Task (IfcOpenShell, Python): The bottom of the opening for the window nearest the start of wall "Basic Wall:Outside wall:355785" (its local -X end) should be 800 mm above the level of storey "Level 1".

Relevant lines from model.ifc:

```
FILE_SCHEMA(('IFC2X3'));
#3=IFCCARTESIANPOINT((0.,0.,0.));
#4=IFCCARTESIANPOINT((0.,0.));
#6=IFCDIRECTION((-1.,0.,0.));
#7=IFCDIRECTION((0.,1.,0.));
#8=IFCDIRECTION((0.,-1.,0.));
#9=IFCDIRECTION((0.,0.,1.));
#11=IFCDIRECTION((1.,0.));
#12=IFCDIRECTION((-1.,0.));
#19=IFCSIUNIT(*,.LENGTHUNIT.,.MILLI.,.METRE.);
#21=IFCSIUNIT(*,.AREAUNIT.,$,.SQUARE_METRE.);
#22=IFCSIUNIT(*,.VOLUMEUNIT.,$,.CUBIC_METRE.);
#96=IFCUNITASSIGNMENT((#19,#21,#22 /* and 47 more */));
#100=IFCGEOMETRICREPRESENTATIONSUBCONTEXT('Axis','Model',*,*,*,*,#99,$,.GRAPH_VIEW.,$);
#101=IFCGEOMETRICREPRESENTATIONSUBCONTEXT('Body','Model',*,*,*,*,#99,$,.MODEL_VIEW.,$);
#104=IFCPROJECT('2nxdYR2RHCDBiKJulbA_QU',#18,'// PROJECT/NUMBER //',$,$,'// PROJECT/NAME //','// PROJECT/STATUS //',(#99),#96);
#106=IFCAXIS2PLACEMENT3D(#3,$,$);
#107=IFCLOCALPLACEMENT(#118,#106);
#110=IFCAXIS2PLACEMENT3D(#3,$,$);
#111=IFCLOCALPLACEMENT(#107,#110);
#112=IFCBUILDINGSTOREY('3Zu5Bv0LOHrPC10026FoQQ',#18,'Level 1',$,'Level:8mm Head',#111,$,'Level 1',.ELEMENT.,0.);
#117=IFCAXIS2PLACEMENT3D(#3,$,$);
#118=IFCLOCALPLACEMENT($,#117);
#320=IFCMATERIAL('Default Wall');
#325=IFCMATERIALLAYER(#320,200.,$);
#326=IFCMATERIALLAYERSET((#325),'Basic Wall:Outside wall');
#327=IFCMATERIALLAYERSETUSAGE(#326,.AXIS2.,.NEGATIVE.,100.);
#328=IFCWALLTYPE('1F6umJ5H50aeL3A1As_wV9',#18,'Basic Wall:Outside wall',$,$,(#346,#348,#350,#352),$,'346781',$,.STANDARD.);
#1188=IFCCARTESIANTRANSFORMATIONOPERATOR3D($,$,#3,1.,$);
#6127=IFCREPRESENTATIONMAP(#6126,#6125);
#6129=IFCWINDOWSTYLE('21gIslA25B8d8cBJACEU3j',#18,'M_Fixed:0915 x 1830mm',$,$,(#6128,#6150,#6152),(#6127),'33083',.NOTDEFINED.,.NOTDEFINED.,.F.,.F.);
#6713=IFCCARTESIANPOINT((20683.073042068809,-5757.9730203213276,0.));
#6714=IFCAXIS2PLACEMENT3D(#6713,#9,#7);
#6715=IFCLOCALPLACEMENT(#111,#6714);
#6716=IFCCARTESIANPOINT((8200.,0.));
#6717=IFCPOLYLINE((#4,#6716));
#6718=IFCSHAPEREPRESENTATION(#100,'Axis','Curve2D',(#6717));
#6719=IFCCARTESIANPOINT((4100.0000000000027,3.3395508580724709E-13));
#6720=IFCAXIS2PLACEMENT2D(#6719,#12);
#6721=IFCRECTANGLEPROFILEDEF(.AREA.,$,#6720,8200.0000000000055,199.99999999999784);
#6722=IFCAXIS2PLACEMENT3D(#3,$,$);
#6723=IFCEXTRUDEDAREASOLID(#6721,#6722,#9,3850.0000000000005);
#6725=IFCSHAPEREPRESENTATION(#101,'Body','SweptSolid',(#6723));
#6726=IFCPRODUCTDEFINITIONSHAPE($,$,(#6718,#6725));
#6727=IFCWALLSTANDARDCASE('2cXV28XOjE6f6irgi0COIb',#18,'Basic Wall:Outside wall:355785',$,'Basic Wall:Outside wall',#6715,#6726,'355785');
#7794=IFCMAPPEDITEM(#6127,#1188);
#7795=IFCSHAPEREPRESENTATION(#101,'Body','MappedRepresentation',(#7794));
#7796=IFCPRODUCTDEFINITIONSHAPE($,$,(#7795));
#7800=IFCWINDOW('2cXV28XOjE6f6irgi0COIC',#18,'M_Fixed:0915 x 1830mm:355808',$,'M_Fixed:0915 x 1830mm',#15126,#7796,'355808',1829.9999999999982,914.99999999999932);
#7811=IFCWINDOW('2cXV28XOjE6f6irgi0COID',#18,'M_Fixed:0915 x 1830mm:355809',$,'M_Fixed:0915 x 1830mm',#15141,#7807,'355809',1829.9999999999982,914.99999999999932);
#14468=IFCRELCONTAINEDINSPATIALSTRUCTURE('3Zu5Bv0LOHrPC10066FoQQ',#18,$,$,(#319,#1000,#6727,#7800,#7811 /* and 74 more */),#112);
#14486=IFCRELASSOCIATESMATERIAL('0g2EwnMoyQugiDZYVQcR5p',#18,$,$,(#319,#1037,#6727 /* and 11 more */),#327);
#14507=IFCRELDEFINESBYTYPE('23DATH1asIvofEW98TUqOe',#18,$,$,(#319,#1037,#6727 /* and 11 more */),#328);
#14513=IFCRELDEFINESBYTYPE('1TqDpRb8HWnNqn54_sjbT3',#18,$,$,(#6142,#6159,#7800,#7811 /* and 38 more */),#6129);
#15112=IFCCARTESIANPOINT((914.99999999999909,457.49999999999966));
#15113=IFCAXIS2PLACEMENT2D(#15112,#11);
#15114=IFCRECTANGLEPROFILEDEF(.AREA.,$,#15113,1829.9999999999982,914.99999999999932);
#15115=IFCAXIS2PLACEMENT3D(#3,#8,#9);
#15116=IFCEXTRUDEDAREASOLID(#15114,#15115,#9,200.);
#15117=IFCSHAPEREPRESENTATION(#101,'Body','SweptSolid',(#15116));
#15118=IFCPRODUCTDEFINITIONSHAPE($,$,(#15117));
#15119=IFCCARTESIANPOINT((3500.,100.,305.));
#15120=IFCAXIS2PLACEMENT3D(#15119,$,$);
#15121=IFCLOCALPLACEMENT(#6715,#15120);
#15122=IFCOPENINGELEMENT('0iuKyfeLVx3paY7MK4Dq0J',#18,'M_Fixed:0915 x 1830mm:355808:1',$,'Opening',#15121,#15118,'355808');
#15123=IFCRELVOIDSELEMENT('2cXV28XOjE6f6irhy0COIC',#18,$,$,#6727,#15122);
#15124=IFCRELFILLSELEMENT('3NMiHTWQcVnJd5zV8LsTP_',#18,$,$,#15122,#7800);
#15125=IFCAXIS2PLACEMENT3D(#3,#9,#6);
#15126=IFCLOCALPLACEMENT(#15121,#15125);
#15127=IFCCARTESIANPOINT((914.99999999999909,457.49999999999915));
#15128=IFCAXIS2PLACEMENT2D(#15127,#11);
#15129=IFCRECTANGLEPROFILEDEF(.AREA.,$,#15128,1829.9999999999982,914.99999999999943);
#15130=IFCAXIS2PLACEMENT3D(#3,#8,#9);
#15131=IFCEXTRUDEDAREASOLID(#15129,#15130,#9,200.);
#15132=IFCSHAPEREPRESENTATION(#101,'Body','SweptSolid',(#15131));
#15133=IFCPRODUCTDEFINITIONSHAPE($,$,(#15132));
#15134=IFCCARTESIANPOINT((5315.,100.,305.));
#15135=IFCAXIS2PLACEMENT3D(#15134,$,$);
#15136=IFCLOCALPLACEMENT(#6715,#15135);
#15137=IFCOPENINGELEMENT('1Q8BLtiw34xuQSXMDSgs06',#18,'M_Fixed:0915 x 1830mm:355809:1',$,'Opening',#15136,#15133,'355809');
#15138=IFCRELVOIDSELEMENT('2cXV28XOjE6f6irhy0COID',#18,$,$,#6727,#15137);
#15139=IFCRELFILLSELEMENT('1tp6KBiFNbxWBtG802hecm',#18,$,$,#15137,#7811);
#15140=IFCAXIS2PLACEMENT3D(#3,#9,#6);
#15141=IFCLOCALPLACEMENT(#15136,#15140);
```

```python
import numpy as np
import ifcopenshell
import ifcopenshell.api.geometry
import ifcopenshell.geom
import ifcopenshell.util.element
import ifcopenshell.util.placement
import ifcopenshell.util.shape
import ifcopenshell.util.unit

model = ifcopenshell.open("model.ifc")
unit_scale = ifcopenshell.util.unit.calculate_unit_scale(model)

window = model.by_guid("2cXV28XOjE6f6irgi0COIC")
opening = window.FillsVoids[0].RelatingOpeningElement
storey = ifcopenshell.util.element.get_container(window, ifc_class="IfcBuildingStorey")
level = ifcopenshell.util.placement.get_local_placement(storey.ObjectPlacement)[2, 3]

# The opening's origin need not be at the sill, so measure its lowest point.
shape = ifcopenshell.geom.create_shape(ifcopenshell.geom.settings(), opening)
bottom = ifcopenshell.util.shape.get_shape_bottom_elevation(shape, shape.geometry) / unit_scale
dz = level + 0.8 / unit_scale - bottom

shift = np.array([0.0, 0.0, dz])
# The window is placed relative to its opening, so it follows when the opening moves.
matrix = ifcopenshell.util.placement.get_local_placement(opening.ObjectPlacement)
matrix[:3, 3] += shift
ifcopenshell.api.geometry.edit_object_placement(
    model, product=opening, matrix=matrix, is_si=False, should_transform_children=True
)

print(f"moved by {dz * unit_scale:+.3f} m")

model.write("model-out.ifc")
```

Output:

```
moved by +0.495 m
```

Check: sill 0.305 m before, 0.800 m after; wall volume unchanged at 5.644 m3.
